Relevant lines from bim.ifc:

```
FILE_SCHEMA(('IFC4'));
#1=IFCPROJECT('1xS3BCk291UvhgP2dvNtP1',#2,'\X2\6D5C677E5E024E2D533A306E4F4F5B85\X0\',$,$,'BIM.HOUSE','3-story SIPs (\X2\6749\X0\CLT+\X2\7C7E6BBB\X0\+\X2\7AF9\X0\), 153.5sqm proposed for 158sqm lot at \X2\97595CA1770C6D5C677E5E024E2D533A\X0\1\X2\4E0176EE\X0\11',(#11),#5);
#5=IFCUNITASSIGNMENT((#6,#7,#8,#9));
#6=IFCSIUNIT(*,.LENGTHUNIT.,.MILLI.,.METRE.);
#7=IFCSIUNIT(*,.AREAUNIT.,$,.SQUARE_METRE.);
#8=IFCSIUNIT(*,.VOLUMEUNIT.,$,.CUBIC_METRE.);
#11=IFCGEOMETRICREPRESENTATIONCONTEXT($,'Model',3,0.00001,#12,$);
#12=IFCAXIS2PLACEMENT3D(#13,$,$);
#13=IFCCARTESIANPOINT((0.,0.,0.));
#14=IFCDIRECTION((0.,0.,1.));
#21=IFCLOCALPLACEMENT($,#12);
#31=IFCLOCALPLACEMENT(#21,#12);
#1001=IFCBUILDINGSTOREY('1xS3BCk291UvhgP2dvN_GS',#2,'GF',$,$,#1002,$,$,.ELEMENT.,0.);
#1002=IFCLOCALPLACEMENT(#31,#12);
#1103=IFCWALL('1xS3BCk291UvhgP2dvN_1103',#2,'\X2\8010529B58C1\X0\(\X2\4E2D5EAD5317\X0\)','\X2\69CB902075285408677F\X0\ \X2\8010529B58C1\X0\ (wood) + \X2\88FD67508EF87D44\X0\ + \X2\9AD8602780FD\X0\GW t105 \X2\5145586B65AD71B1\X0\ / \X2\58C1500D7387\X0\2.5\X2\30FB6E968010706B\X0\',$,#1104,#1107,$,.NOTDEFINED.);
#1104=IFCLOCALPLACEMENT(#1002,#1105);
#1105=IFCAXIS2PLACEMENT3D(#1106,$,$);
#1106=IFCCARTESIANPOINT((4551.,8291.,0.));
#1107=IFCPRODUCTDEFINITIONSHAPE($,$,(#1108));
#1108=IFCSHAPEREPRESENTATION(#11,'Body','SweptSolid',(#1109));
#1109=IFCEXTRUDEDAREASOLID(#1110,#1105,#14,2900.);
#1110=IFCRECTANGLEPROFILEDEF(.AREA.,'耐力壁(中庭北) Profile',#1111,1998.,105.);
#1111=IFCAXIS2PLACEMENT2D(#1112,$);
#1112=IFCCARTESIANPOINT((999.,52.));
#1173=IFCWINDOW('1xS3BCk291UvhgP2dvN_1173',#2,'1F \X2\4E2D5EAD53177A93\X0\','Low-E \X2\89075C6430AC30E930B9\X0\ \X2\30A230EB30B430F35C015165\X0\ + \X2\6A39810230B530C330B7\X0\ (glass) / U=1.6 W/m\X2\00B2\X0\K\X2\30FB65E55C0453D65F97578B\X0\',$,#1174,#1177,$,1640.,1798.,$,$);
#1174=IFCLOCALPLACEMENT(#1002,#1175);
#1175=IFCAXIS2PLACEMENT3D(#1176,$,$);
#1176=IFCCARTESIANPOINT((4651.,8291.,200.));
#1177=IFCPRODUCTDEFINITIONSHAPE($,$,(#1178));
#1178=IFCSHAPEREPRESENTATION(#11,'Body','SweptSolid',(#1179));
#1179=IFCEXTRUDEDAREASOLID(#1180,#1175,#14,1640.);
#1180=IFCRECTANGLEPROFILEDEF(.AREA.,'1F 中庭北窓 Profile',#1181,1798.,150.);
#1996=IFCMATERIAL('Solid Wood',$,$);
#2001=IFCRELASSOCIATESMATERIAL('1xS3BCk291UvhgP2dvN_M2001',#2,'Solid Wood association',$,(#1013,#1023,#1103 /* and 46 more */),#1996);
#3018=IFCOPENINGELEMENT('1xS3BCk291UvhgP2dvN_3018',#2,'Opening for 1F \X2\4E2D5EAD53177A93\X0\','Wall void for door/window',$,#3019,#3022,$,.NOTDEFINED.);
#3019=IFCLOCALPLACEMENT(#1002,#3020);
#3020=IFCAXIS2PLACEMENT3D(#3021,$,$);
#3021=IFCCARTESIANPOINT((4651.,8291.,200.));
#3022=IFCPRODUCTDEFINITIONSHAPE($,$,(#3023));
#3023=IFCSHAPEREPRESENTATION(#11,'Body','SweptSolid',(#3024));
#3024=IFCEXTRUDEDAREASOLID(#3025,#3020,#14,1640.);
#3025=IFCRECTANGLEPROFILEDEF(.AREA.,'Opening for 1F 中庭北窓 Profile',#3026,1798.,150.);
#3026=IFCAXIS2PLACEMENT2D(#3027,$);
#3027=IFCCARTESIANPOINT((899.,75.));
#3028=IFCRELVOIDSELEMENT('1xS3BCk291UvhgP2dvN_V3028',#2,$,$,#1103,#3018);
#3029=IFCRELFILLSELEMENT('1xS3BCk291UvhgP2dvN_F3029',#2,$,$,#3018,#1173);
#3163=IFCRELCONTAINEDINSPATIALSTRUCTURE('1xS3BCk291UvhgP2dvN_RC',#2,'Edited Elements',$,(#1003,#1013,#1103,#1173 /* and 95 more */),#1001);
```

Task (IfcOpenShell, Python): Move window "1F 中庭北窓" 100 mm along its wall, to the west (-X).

```python
import ifcopenshell
import ifcopenshell.api.geometry
import ifcopenshell.util.placement
import ifcopenshell.util.unit

model = ifcopenshell.open("bim.ifc")
unit_scale = ifcopenshell.util.unit.calculate_unit_scale(model)

window = model.by_guid("1xS3BCk291UvhgP2dvN_1173")
opening = window.FillsVoids[0].RelatingOpeningElement
wall = opening.VoidsElements[0].RelatingBuildingElement

wall_matrix = ifcopenshell.util.placement.get_local_placement(wall.ObjectPlacement)
shift = wall_matrix[:3, 0] * -0.1 / unit_scale
before = ifcopenshell.util.placement.get_local_placement(window.ObjectPlacement)[:3, 3].copy()

# The window is not placed relative to its opening, so move both.
for product in (opening, window):
    matrix = ifcopenshell.util.placement.get_local_placement(product.ObjectPlacement)
    matrix[:3, 3] += shift
    ifcopenshell.api.geometry.edit_object_placement(model, product=product, matrix=matrix, is_si=False)

after = ifcopenshell.util.placement.get_local_placement(window.ObjectPlacement)[:3, 3]
print("window moved by", (after - before).round(3) + 0.0)

model.write("bim_updated.ifc")
```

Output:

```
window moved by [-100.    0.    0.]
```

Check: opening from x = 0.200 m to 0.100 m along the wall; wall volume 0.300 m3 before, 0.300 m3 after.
